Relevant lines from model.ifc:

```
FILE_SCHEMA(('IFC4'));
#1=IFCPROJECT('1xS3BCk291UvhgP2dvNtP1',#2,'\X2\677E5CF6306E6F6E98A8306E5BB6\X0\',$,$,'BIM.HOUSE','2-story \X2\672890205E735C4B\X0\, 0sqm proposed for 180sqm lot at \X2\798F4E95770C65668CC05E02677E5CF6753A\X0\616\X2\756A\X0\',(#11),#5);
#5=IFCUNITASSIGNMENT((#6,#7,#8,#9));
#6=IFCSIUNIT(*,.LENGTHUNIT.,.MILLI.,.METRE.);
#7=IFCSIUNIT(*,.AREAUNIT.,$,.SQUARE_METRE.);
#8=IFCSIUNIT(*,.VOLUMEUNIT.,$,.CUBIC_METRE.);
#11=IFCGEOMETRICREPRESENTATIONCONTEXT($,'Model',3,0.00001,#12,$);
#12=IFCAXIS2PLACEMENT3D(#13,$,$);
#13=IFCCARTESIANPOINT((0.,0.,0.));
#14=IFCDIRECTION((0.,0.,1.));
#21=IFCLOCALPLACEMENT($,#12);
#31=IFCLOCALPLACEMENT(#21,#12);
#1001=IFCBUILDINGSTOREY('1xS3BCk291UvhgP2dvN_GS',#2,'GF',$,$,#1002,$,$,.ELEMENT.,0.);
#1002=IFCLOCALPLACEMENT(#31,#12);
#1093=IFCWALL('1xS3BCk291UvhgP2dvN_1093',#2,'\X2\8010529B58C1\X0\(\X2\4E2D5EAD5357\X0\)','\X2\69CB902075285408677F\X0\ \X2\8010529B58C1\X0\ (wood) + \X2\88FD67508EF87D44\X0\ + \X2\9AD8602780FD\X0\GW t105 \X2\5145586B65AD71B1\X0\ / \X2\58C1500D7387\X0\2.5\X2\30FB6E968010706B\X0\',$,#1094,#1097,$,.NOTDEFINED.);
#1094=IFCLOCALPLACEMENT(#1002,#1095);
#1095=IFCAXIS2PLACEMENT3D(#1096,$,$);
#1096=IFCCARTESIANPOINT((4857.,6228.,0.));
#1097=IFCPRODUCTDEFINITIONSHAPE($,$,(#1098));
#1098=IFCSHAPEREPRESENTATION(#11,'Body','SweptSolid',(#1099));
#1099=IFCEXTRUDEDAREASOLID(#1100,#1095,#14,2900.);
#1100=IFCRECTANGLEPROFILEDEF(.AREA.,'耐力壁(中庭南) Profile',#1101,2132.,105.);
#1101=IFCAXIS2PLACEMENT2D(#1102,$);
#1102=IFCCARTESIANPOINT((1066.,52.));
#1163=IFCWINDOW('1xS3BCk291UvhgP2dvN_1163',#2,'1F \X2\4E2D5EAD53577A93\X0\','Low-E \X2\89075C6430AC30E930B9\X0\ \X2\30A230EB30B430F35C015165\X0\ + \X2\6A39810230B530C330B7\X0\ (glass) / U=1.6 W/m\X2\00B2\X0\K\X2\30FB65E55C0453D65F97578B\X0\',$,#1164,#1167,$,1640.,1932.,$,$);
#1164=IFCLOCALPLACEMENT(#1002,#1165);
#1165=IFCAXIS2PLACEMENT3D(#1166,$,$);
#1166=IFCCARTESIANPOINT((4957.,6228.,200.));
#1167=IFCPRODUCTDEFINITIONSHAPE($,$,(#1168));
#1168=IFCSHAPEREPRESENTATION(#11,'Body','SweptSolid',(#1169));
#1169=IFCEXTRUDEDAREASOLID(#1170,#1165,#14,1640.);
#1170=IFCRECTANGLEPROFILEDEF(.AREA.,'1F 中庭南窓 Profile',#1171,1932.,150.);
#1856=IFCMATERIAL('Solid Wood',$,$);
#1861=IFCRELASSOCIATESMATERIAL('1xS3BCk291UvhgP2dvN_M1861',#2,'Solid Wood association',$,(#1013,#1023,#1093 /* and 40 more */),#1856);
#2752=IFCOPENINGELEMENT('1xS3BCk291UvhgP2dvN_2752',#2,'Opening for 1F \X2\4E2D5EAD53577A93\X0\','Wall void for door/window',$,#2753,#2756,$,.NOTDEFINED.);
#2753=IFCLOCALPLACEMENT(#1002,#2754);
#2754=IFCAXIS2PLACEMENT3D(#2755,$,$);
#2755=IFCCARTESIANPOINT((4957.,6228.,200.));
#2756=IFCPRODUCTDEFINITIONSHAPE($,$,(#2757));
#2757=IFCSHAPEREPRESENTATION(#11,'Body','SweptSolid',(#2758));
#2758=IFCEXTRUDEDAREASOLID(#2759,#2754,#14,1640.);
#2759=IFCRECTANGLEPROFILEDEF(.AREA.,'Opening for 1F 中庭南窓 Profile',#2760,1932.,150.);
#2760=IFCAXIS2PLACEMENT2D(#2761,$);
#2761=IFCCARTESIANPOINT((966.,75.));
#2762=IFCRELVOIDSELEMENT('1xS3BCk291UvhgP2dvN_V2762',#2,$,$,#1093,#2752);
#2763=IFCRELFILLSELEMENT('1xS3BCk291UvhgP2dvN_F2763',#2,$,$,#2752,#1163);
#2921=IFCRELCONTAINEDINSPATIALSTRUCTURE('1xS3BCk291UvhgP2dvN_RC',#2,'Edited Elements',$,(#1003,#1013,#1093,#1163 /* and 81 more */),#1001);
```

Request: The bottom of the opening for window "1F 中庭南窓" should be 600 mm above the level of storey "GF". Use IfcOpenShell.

```python
import numpy as np
import ifcopenshell
import ifcopenshell.api.geometry
import ifcopenshell.geom
import ifcopenshell.util.element
import ifcopenshell.util.placement
import ifcopenshell.util.shape
import ifcopenshell.util.unit

model = ifcopenshell.open("model.ifc")
unit_scale = ifcopenshell.util.unit.calculate_unit_scale(model)

window = model.by_id(1163)
opening = window.FillsVoids[0].RelatingOpeningElement
storey = ifcopenshell.util.element.get_container(window, ifc_class="IfcBuildingStorey")
level = ifcopenshell.util.placement.get_local_placement(storey.ObjectPlacement)[2, 3]

# The opening's origin need not be at the sill, so measure its lowest point.
shape = ifcopenshell.geom.create_shape(ifcopenshell.geom.settings(), opening)
bottom = ifcopenshell.util.shape.get_shape_bottom_elevation(shape, shape.geometry) / unit_scale
dz = level + 0.6 / unit_scale - bottom

shift = np.array([0.0, 0.0, dz])
# The window is not placed relative to its opening, so move both.
for product in (opening, window):
    matrix = ifcopenshell.util.placement.get_local_placement(product.ObjectPlacement)
    matrix[:3, 3] += shift
    ifcopenshell.api.geometry.edit_object_placement(model, product=product, matrix=matrix, is_si=False)

print(f"moved by {dz * unit_scale:+.3f} m")

model.write("model_rev.ifc")
```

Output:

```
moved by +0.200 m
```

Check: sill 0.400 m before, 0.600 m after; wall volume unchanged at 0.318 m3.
